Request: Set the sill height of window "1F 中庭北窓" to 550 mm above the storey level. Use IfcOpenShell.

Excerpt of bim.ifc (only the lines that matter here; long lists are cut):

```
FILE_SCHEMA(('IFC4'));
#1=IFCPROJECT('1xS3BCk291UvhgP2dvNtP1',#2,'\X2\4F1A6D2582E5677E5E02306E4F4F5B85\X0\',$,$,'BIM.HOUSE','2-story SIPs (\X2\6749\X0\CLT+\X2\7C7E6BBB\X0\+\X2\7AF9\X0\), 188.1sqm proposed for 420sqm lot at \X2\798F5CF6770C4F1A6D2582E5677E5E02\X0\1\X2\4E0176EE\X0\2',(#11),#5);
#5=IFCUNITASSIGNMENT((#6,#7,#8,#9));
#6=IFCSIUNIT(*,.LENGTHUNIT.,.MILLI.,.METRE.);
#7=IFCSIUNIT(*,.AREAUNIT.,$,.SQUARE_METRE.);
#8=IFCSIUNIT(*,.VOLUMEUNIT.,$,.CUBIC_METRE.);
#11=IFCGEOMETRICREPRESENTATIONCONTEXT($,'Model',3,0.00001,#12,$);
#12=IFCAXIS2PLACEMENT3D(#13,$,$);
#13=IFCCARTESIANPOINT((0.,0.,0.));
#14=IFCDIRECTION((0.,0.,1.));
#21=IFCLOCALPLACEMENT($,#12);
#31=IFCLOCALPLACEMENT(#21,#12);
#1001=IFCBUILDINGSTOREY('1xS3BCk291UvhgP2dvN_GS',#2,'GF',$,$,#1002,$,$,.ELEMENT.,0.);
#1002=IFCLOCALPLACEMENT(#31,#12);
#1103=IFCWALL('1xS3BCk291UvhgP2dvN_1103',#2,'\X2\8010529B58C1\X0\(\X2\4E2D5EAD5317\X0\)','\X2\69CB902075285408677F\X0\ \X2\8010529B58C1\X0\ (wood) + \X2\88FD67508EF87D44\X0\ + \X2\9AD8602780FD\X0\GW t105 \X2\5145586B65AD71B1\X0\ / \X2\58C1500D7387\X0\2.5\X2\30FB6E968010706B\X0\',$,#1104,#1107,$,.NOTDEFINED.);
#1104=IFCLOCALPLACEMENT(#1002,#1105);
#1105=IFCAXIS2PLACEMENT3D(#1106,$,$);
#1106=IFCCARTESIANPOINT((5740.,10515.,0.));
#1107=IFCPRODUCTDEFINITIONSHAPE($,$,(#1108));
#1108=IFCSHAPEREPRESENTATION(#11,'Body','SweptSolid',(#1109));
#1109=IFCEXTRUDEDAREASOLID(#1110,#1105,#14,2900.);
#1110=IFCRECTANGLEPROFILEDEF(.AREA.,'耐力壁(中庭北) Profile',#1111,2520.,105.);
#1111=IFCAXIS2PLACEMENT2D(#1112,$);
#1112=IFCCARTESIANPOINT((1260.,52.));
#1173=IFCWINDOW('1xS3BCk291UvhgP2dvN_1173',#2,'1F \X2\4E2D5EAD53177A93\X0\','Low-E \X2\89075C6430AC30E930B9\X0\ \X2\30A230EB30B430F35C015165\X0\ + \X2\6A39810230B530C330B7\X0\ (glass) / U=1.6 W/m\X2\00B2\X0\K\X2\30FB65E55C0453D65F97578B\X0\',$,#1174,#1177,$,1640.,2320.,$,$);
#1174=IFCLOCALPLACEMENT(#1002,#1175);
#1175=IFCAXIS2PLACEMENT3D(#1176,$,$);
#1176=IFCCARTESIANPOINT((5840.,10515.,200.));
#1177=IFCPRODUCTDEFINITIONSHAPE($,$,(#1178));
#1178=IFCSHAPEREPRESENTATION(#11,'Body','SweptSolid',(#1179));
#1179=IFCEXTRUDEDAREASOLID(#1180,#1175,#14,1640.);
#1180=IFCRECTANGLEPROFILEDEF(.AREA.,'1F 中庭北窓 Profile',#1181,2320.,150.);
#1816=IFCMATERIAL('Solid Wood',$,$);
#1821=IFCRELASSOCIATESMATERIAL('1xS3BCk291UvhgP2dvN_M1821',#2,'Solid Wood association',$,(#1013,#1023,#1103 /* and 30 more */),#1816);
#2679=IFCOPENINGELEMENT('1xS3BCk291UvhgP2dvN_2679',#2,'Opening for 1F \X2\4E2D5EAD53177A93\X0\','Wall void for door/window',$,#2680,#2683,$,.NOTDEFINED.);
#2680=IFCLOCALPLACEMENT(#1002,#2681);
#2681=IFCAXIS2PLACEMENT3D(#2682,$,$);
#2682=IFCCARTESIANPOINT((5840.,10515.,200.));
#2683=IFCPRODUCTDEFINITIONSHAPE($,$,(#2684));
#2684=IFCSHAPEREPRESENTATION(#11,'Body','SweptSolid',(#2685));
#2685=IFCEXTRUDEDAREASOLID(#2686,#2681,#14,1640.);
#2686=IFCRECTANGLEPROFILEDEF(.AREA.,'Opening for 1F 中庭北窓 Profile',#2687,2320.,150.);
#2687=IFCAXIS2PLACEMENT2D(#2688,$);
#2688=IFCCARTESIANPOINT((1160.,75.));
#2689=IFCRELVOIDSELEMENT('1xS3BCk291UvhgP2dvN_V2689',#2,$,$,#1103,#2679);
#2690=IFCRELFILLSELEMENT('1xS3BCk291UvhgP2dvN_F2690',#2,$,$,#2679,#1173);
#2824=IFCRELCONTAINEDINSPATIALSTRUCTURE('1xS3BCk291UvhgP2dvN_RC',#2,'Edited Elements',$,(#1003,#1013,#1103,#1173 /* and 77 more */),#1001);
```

```python
import numpy as np
import ifcopenshell
import ifcopenshell.api.geometry
import ifcopenshell.geom
import ifcopenshell.util.element
import ifcopenshell.util.placement
import ifcopenshell.util.shape
import ifcopenshell.util.unit

model = ifcopenshell.open("bim.ifc")
unit_scale = ifcopenshell.util.unit.calculate_unit_scale(model)

window = model.by_guid("1xS3BCk291UvhgP2dvN_1173")
opening = window.FillsVoids[0].RelatingOpeningElement
storey = ifcopenshell.util.element.get_container(window, ifc_class="IfcBuildingStorey")
level = ifcopenshell.util.placement.get_local_placement(storey.ObjectPlacement)[2, 3]

# The opening's origin need not be at the sill, so measure its lowest point.
shape = ifcopenshell.geom.create_shape(ifcopenshell.geom.settings(), opening)
bottom = ifcopenshell.util.shape.get_shape_bottom_elevation(shape, shape.geometry) / unit_scale
dz = level + 0.55 / unit_scale - bottom

shift = np.array([0.0, 0.0, dz])
# The window is not placed relative to its opening, so move both.
for product in (opening, window):
    matrix = ifcopenshell.util.placement.get_local_placement(product.ObjectPlacement)
    matrix[:3, 3] += shift
    ifcopenshell.api.geometry.edit_object_placement(model, product=product, matrix=matrix, is_si=False)

print(f"moved by {dz * unit_scale:+.3f} m")

model.write("bim-out.ifc")
```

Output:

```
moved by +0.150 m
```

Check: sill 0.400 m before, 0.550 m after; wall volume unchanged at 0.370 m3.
